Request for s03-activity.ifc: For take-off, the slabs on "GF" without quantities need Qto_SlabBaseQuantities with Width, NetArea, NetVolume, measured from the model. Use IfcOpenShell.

First a look at what the model holds.

```python
import ifcopenshell
import ifcopenshell.util.element
import ifcopenshell.util.unit

model = ifcopenshell.open("s03-activity.ifc")
print(model.schema)
for unit_type in ("LENGTHUNIT", "AREAUNIT", "VOLUMEUNIT"):
    print(unit_type, ifcopenshell.util.unit.calculate_unit_scale(model, unit_type))
storey = next(s for s in model.by_type("IfcBuildingStorey") if s.Name == "GF")
slabs = [e for e in ifcopenshell.util.element.get_decomposition(storey) if e.is_a("IfcSlab")]
for e in sorted(slabs, key=lambda e: e.id()):
    print(e.id(), e.is_a(), e.Name, list(ifcopenshell.util.element.get_psets(e, qtos_only=True)), sep=" | ")
```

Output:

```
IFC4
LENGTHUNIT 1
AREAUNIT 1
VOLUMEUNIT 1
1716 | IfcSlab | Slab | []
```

```python
import ifcopenshell
import ifcopenshell.api.pset
import ifcopenshell.geom
import ifcopenshell.util.element
import ifcopenshell.util.shape
import ifcopenshell.util.unit

model = ifcopenshell.open("s03-activity.ifc")
unit_scale = ifcopenshell.util.unit.calculate_unit_scale(model)
area_scale = ifcopenshell.util.unit.calculate_unit_scale(model, "AREAUNIT")
volume_scale = ifcopenshell.util.unit.calculate_unit_scale(model, "VOLUMEUNIT")
settings = ifcopenshell.geom.settings()

storey = next(s for s in model.by_type("IfcBuildingStorey") if s.Name == "GF")
slabs = [e for e in ifcopenshell.util.element.get_decomposition(storey) if e.is_a("IfcSlab")]

for e in sorted(slabs, key=lambda e: e.id()):
    if ifcopenshell.util.element.get_psets(e, qtos_only=True, should_inherit=False):
        continue
    # Geometry comes back in metres, in the element's own axes.
    shape = ifcopenshell.geom.create_shape(settings, e)
    values = {
        "Width": ifcopenshell.util.shape.get_z(shape.geometry) / unit_scale,
        "NetArea": ifcopenshell.util.shape.get_footprint_area(shape.geometry) / area_scale,
        "NetVolume": ifcopenshell.util.shape.get_volume(shape.geometry) / volume_scale,
    }
    qto = ifcopenshell.api.pset.add_qto(model, product=e, name="Qto_SlabBaseQuantities")
    ifcopenshell.api.pset.edit_qto(model, qto=qto, properties=values)
    print(e.id(), {k: round(v, 3) for k, v in values.items()})

model.write("s03-activity_edited.ifc")
```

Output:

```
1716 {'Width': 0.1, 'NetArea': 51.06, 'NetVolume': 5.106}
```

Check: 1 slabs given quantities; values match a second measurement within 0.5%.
